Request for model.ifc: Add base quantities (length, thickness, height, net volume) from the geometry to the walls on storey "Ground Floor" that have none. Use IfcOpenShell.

First a look at what the model holds.

```python
import ifcopenshell
import ifcopenshell.util.element
import ifcopenshell.util.unit

model = ifcopenshell.open("model.ifc")
print(model.schema)
for unit_type in ("LENGTHUNIT", "AREAUNIT", "VOLUMEUNIT"):
    print(unit_type, ifcopenshell.util.unit.calculate_unit_scale(model, unit_type))
storey = next(s for s in model.by_type("IfcBuildingStorey") if s.Name == "Ground Floor")
walls = [e for e in ifcopenshell.util.element.get_decomposition(storey) if e.is_a("IfcWall")]
for e in sorted(walls, key=lambda e: e.id()):
    print(e.id(), e.is_a(), e.Name, list(ifcopenshell.util.element.get_psets(e, qtos_only=True)), sep=" | ")
```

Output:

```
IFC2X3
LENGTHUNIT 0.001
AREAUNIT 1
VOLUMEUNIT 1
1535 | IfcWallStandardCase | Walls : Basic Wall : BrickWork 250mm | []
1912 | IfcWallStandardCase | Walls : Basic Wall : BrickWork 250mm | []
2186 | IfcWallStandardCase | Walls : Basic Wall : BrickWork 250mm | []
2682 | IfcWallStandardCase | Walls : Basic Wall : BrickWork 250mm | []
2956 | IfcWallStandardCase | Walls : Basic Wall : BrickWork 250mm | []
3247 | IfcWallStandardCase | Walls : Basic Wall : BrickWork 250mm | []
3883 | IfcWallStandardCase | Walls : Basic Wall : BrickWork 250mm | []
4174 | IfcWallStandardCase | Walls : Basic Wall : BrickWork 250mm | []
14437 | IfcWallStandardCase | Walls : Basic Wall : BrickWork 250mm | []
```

```python
import ifcopenshell
import ifcopenshell.api.pset
import ifcopenshell.geom
import ifcopenshell.util.element
import ifcopenshell.util.shape
import ifcopenshell.util.unit

model = ifcopenshell.open("model.ifc")
unit_scale = ifcopenshell.util.unit.calculate_unit_scale(model)
volume_scale = ifcopenshell.util.unit.calculate_unit_scale(model, "VOLUMEUNIT")
settings = ifcopenshell.geom.settings()

storey = next(s for s in model.by_type("IfcBuildingStorey") if s.Name == "Ground Floor")
walls = [e for e in ifcopenshell.util.element.get_decomposition(storey) if e.is_a("IfcWall")]

for e in sorted(walls, key=lambda e: e.id()):
    if ifcopenshell.util.element.get_psets(e, qtos_only=True, should_inherit=False):
        continue
    # Geometry comes back in metres, in the element's own axes.
    shape = ifcopenshell.geom.create_shape(settings, e)
    values = {
        "Length": ifcopenshell.util.shape.get_x(shape.geometry) / unit_scale,
        "Width": ifcopenshell.util.shape.get_y(shape.geometry) / unit_scale,
        "Height": ifcopenshell.util.shape.get_z(shape.geometry) / unit_scale,
        "NetVolume": ifcopenshell.util.shape.get_volume(shape.geometry) / volume_scale,
    }
    qto = ifcopenshell.api.pset.add_qto(model, product=e, name="BaseQuantities")
    ifcopenshell.api.pset.edit_qto(model, qto=qto, properties=values)
    print(e.id(), {k: round(v, 3) for k, v in values.items()})

model.write("model_rev.ifc")
```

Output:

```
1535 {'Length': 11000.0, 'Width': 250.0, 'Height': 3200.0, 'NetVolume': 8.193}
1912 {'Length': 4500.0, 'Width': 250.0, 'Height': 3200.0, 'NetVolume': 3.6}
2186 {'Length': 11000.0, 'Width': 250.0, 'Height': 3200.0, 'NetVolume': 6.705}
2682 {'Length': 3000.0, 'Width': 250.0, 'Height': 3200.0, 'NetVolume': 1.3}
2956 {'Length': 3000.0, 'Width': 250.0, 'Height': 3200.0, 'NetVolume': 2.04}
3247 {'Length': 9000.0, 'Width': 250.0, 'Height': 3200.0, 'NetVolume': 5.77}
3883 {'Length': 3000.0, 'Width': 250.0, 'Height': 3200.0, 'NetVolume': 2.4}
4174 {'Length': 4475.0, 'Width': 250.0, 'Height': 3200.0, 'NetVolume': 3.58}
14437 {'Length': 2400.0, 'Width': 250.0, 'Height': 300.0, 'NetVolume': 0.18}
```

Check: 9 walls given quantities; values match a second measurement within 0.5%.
